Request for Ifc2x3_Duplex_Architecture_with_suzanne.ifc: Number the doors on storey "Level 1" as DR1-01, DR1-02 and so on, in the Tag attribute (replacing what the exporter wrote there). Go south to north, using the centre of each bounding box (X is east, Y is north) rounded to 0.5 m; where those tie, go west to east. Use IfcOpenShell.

First a look at what the model holds.

```python
import ifcopenshell
import ifcopenshell.util.element
import ifcopenshell.util.placement

model = ifcopenshell.open("Ifc2x3_Duplex_Architecture_with_suzanne.ifc")
print(model.schema)
storey = next(s for s in model.by_type("IfcBuildingStorey") if s.Name == "Level 1")
doors = [e for e in ifcopenshell.util.element.get_decomposition(storey) if e.is_a("IfcDoor")]
for e in sorted(doors, key=lambda e: e.id()):
    origin = ifcopenshell.util.placement.get_local_placement(e.ObjectPlacement)[:3, 3]
    print(e.id(), e.Tag, e.Name, origin.round(2) + 0.0, sep=" | ")
```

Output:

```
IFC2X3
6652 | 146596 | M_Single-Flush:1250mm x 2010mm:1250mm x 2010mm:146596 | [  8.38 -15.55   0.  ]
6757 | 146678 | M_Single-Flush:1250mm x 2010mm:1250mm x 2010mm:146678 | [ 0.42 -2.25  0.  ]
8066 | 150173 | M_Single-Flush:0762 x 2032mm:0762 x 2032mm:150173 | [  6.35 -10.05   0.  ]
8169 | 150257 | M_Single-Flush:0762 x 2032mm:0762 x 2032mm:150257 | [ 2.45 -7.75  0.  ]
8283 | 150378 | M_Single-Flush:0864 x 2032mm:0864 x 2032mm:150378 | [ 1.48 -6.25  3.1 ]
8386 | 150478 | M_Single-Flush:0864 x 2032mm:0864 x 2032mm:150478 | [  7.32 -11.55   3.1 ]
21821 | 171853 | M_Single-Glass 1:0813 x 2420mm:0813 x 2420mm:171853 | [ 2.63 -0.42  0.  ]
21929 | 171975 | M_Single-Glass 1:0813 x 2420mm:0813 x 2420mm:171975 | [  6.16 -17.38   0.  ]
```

```python
import ifcopenshell
import ifcopenshell.geom
import ifcopenshell.util.element
import ifcopenshell.util.shape

model = ifcopenshell.open("Ifc2x3_Duplex_Architecture_with_suzanne.ifc")
settings = ifcopenshell.geom.settings()
settings.set("use-world-coords", True)


def centre(element):
    shape = ifcopenshell.geom.create_shape(settings, element)
    return ifcopenshell.util.shape.get_bbox_centroid(shape.geometry)


storey = next(s for s in model.by_type("IfcBuildingStorey") if s.Name == "Level 1")
doors = [e for e in ifcopenshell.util.element.get_decomposition(storey) if e.is_a("IfcDoor")]

# Insertion points can sit at a corner or the storey origin, so sort by the geometry (in metres).
centres = {e: centre(e) for e in doors}
doors.sort(key=lambda e: (round(centres[e][1] / 0.5), centres[e][0]))

for i, e in enumerate(doors, start=1):
    number = f"DR1-{i:02d}"
    e.Tag = number
    print(e.id(), number)

model.write("Ifc2x3_Duplex_Architecture_with_suzanne_v2.ifc")
```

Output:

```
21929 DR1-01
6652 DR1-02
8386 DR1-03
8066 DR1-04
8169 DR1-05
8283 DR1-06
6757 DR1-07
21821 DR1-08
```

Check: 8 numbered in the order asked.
